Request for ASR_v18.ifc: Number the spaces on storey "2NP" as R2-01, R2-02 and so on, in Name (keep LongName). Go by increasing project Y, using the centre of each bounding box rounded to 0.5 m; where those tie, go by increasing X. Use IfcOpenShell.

First a look at what the model holds.

```python
import ifcopenshell
import ifcopenshell.util.element
import ifcopenshell.util.placement

model = ifcopenshell.open("ASR_v18.ifc")
print(model.schema)
storey = next(s for s in model.by_type("IfcBuildingStorey") if s.Name == "2NP")
spaces = [e for e in ifcopenshell.util.element.get_decomposition(storey) if e.is_a("IfcSpace")]
for e in sorted(spaces, key=lambda e: e.id()):
    origin = ifcopenshell.util.placement.get_local_placement(e.ObjectPlacement)[:3, 3]
    print(e.id(), e.Name, e.LongName, origin.round(2) + 0.0, sep=" | ")
```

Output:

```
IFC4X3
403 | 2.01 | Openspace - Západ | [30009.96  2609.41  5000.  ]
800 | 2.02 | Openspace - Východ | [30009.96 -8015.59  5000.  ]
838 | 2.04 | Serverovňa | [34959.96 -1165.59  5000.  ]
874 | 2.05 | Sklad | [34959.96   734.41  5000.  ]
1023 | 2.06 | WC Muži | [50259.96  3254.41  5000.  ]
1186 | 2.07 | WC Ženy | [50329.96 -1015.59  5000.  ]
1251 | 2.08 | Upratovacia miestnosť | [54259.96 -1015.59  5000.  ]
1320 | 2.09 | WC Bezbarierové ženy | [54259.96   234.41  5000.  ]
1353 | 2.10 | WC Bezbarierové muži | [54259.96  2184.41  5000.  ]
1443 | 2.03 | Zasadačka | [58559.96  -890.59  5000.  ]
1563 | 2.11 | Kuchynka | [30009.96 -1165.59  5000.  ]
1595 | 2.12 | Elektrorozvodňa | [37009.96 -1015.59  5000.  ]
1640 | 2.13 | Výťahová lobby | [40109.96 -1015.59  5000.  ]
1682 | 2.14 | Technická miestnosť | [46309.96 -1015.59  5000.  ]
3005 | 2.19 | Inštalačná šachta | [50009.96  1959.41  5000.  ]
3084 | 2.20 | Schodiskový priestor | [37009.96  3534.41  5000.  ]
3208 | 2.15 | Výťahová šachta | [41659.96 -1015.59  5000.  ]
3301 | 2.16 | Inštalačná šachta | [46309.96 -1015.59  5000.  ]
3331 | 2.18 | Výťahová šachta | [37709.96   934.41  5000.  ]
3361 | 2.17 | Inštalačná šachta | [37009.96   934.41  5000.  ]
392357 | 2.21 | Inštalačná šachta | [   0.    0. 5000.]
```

```python
import ifcopenshell
import ifcopenshell.geom
import ifcopenshell.util.element
import ifcopenshell.util.shape

model = ifcopenshell.open("ASR_v18.ifc")
settings = ifcopenshell.geom.settings()
settings.set("use-world-coords", True)


def centre(element):
    shape = ifcopenshell.geom.create_shape(settings, element)
    return ifcopenshell.util.shape.get_bbox_centroid(shape.geometry)


storey = next(s for s in model.by_type("IfcBuildingStorey") if s.Name == "2NP")
spaces = [e for e in ifcopenshell.util.element.get_decomposition(storey) if e.is_a("IfcSpace")]

# Insertion points can sit at a corner or the storey origin, so sort by the geometry (in metres).
centres = {e: centre(e) for e in spaces}
spaces.sort(key=lambda e: (round(centres[e][1] / 0.5), centres[e][0]))

for i, e in enumerate(spaces, start=1):
    number = f"R2-{i:02d}"
    e.Name = number
    print(e.id(), number)

model.write("ASR_v18_rev.ifc")
```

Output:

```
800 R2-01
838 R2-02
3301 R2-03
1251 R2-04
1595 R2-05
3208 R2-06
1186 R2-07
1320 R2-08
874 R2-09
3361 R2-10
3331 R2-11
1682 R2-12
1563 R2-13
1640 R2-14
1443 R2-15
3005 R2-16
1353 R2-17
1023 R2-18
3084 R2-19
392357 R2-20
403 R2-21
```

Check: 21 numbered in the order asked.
